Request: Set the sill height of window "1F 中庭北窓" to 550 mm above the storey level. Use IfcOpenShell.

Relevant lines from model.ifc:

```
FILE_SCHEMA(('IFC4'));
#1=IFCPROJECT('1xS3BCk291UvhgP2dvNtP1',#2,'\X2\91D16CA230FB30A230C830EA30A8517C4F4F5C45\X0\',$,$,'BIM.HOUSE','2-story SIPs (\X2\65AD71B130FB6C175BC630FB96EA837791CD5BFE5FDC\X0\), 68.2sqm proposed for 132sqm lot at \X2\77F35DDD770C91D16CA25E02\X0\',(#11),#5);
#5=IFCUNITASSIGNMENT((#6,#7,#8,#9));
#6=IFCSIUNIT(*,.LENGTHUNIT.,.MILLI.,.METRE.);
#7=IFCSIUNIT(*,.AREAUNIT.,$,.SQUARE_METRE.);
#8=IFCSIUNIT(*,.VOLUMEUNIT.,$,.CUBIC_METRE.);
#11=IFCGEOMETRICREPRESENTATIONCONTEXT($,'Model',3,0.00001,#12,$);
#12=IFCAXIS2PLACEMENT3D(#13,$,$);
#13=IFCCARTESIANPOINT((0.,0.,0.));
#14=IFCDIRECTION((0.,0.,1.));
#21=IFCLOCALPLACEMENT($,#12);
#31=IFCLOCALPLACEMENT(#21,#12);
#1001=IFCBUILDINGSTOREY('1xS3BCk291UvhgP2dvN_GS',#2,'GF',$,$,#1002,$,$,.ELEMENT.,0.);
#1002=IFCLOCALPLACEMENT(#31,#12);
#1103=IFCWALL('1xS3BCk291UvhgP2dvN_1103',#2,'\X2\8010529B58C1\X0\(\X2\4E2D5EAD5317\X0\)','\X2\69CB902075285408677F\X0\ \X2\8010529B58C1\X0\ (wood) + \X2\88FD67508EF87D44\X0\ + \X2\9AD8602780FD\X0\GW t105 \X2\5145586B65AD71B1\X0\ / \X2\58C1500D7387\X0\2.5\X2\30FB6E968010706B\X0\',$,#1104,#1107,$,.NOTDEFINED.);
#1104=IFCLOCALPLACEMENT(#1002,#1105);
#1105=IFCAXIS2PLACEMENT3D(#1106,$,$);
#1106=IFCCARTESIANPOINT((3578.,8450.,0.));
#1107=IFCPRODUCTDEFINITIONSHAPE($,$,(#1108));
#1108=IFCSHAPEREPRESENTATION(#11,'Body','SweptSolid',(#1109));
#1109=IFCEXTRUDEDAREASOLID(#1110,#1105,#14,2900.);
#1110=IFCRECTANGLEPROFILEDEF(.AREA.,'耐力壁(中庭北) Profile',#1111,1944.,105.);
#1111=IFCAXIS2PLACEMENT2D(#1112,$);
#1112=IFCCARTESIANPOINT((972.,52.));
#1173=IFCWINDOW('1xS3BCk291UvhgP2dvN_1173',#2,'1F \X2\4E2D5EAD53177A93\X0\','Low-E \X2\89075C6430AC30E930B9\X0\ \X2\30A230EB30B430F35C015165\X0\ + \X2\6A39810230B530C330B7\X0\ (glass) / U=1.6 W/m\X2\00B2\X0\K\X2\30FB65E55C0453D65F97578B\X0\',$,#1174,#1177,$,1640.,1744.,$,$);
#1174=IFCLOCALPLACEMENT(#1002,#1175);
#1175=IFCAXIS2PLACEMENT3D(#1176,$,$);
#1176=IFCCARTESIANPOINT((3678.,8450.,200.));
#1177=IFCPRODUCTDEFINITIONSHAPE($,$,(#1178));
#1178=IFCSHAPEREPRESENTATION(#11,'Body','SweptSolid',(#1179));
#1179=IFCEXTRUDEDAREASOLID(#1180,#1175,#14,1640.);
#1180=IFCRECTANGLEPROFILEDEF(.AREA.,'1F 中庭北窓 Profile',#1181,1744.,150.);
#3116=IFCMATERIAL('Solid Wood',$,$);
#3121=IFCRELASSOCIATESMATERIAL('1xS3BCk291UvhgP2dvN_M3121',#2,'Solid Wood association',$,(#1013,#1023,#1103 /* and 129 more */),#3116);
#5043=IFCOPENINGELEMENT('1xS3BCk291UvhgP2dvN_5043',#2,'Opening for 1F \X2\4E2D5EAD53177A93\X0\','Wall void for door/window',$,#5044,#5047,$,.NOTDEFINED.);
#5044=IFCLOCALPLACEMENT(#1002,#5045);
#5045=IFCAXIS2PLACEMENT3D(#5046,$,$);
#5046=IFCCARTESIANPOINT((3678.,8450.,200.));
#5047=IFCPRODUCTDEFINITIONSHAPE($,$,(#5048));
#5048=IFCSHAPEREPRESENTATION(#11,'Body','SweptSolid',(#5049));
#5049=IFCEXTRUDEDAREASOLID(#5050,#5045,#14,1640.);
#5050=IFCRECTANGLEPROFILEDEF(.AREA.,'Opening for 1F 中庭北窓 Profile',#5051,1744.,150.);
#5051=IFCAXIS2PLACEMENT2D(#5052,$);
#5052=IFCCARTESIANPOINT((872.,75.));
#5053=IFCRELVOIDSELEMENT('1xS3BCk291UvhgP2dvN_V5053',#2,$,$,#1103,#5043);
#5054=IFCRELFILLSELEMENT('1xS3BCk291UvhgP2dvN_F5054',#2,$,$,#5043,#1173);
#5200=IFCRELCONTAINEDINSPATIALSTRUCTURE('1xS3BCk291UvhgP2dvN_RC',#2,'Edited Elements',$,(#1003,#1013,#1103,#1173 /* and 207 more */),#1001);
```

```python
import numpy as np
import ifcopenshell
import ifcopenshell.api.geometry
import ifcopenshell.geom
import ifcopenshell.util.element
import ifcopenshell.util.placement
import ifcopenshell.util.shape
import ifcopenshell.util.unit

model = ifcopenshell.open("model.ifc")
unit_scale = ifcopenshell.util.unit.calculate_unit_scale(model)

window = model.by_guid("1xS3BCk291UvhgP2dvN_1173")
opening = window.FillsVoids[0].RelatingOpeningElement
storey = ifcopenshell.util.element.get_container(window, ifc_class="IfcBuildingStorey")
level = ifcopenshell.util.placement.get_local_placement(storey.ObjectPlacement)[2, 3]

# The opening's origin need not be at the sill, so measure its lowest point.
shape = ifcopenshell.geom.create_shape(ifcopenshell.geom.settings(), opening)
bottom = ifcopenshell.util.shape.get_shape_bottom_elevation(shape, shape.geometry) / unit_scale
dz = level + 550.0 - bottom

shift = np.array([0.0, 0.0, dz])
# The window is not placed relative to its opening, so move both.
for product in (opening, window):
    matrix = ifcopenshell.util.placement.get_local_placement(product.ObjectPlacement)
    matrix[:3, 3] += shift
    ifcopenshell.api.geometry.edit_object_placement(model, product=product, matrix=matrix, is_si=False)

print(f"moved by {dz * unit_scale:+.3f} m")

model.write("model-out.ifc")
```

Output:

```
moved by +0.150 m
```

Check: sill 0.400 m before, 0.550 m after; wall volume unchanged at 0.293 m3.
